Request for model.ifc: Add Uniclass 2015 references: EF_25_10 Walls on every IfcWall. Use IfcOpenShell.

First a look at what the model holds.

```python
import ifcopenshell

model = ifcopenshell.open("model.ifc")
print(model.schema)
print("classifications:", [c.Name for c in model.by_type("IfcClassification")])
for ifc_class in ("IfcDoor", "IfcRoof", "IfcStair", "IfcWall", "IfcWindow"):
    print(ifc_class, len(model.by_type(ifc_class)))
```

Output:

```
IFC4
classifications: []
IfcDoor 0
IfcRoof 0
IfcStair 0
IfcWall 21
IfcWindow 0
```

```python
import ifcopenshell
import ifcopenshell.api.classification

model = ifcopenshell.open("model.ifc")

system = ifcopenshell.api.classification.add_classification(model, classification="Uniclass 2015")

codes = {
    "IfcWall": ("EF_25_10", "Walls"),
}
for ifc_class, (code, name) in codes.items():
    products = model.by_type(ifc_class)
    ifcopenshell.api.classification.add_reference(
        model, products=products, classification=system, identification=code, name=name
    )
    print(code, len(products))

model.write("model-out.ifc")
```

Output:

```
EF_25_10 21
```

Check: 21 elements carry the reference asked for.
